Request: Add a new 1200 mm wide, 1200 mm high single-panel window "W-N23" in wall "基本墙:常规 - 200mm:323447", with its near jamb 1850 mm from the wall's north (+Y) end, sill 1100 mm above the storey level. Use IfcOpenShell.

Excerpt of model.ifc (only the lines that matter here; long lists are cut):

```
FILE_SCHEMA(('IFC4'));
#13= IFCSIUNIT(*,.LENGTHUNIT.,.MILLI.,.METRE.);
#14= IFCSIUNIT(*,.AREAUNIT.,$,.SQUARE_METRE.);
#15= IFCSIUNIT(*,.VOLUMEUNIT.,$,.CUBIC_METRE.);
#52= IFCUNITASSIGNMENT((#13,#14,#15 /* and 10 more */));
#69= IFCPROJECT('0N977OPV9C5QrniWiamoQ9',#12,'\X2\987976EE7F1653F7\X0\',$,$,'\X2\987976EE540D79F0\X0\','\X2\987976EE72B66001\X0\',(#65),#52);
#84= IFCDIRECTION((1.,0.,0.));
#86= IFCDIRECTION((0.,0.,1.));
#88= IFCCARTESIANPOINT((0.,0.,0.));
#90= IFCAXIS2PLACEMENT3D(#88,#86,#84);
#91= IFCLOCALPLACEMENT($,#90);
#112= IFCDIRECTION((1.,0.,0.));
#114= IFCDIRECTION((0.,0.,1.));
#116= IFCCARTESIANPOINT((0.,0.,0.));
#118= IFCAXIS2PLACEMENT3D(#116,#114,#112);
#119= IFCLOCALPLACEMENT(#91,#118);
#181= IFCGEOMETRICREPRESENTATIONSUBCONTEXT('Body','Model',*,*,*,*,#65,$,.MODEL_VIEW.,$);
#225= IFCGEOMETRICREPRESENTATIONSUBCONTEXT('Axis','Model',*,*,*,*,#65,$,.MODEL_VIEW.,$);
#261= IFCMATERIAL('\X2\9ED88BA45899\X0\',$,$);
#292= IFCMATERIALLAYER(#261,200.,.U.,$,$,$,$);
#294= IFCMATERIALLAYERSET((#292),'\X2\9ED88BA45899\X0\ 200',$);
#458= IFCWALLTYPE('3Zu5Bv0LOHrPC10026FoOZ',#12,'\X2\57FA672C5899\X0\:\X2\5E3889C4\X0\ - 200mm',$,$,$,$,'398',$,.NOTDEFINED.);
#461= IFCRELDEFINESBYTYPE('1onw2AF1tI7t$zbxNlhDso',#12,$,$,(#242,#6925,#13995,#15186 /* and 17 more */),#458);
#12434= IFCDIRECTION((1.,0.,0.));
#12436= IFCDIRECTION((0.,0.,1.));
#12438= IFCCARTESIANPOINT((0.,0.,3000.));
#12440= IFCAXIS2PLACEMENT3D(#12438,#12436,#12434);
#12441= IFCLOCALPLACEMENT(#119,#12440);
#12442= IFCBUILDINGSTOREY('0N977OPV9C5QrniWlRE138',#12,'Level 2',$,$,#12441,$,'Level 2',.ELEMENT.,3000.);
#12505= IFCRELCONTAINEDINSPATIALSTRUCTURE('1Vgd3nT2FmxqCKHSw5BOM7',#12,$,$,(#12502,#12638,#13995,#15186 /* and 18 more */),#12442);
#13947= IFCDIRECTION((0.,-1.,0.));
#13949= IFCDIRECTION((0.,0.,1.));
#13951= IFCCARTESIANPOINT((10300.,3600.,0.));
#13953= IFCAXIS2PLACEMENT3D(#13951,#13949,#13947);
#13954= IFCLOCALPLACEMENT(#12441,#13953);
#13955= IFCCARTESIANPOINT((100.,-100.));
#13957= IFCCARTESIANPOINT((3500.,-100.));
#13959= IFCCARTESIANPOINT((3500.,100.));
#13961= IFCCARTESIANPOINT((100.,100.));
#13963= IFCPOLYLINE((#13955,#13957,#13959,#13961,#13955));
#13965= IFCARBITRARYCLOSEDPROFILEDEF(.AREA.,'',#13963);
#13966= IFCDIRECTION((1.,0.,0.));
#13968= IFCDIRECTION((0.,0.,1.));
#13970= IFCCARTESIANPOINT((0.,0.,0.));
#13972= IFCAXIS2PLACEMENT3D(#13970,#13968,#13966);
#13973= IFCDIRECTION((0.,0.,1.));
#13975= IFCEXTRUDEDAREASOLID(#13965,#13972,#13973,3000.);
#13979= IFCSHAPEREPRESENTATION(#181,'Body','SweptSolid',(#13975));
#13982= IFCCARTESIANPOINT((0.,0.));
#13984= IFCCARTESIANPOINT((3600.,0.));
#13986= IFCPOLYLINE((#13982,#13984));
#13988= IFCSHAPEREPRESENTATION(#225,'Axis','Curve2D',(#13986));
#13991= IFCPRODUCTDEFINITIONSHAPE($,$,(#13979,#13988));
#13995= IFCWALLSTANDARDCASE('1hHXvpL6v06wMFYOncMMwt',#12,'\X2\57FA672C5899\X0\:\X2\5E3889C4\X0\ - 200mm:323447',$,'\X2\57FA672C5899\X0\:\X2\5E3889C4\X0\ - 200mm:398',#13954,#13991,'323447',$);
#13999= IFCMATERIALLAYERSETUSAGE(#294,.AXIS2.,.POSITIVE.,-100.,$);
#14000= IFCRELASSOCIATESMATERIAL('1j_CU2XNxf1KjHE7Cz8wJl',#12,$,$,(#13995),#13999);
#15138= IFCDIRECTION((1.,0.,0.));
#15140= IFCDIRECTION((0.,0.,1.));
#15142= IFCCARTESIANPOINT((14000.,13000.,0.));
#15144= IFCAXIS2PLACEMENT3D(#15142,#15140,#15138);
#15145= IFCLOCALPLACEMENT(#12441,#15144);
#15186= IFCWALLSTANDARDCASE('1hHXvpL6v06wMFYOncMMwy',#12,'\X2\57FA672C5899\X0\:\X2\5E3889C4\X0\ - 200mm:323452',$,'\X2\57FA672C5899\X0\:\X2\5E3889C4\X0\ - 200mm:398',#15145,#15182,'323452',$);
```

```python
import numpy as np
import ifcopenshell
import ifcopenshell.api.feature
import ifcopenshell.api.geometry
import ifcopenshell.api.root
import ifcopenshell.api.spatial
import ifcopenshell.geom
import ifcopenshell.util.element
import ifcopenshell.util.placement
import ifcopenshell.util.representation
import ifcopenshell.util.shape
import ifcopenshell.util.unit

model = ifcopenshell.open("model.ifc")
unit_scale = ifcopenshell.util.unit.calculate_unit_scale(model)
settings = ifcopenshell.geom.settings()


def volume(element):
    """Net volume in cubic metres, openings subtracted."""
    shape = ifcopenshell.geom.create_shape(settings, element)
    return ifcopenshell.util.shape.get_volume(shape.geometry)


wall = model.by_guid("1hHXvpL6v06wMFYOncMMwt")
storey = ifcopenshell.util.element.get_container(wall, ifc_class="IfcBuildingStorey")
context = ifcopenshell.util.representation.get_context(model, "Model", "Body", "MODEL_VIEW")
before = volume(wall)

width, height, from_end, sill = 1.2, 1.2, 1.85, 1.1  # metres

# The wall runs along its own X axis, and the end named is its -X end.
wall_shape = ifcopenshell.geom.create_shape(settings, wall)
x, y, z = ifcopenshell.util.shape.get_vertices(wall_shape.geometry).T
start = x.min() + from_end
face, thickness = float(y.min()), float(y.max() - y.min())
wall_matrix = ifcopenshell.util.placement.get_local_placement(wall.ObjectPlacement)
level = ifcopenshell.util.placement.get_local_placement(storey.ObjectPlacement)[2, 3]


def in_wall(x, y):
    """Placement at x, y metres in the wall's axes, at sill height."""
    matrix = wall_matrix.copy()
    matrix[:, 3] = wall_matrix @ np.array([x / unit_scale, y / unit_scale, 0.0, 1.0])
    matrix[2, 3] = level + sill / unit_scale
    return matrix


# Opening: a box that overshoots both wall faces by 50 mm.
opening = ifcopenshell.api.root.create_entity(model, ifc_class="IfcOpeningElement", predefined_type="OPENING")
box = ifcopenshell.api.geometry.add_wall_representation(
    model, context=context, length=width, height=height, thickness=thickness + 0.1
)
ifcopenshell.api.geometry.assign_representation(model, product=opening, representation=box)
ifcopenshell.api.geometry.edit_object_placement(model, product=opening, matrix=in_wall(start, face - 0.05), is_si=False)
ifcopenshell.api.feature.add_feature(model, feature=opening, element=wall)

window = ifcopenshell.api.root.create_entity(model, ifc_class="IfcWindow", name="W-N23", predefined_type="WINDOW")
window.OverallWidth, window.OverallHeight = width / unit_scale, height / unit_scale
window.PartitioningType = "SINGLE_PANEL"
body = ifcopenshell.api.geometry.add_window_representation(
    model,
    context=context,
    overall_width=window.OverallWidth,
    overall_height=window.OverallHeight,
    partition_type="SINGLE_PANEL",
)
ifcopenshell.api.geometry.assign_representation(model, product=window, representation=body)
ifcopenshell.api.spatial.assign_container(model, products=[window], relating_structure=storey)
ifcopenshell.api.feature.add_filling(model, opening=opening, element=window)

# Centre the window in the wall's thickness.
ifcopenshell.api.geometry.edit_object_placement(model, product=window, matrix=in_wall(start, face), is_si=False)
window_shape = ifcopenshell.geom.create_shape(settings, window)
depth = ifcopenshell.util.shape.get_vertices(window_shape.geometry)[:, 1]
offset = face + thickness / 2 - (depth.min() + depth.max()) / 2
ifcopenshell.api.geometry.edit_object_placement(model, product=window, matrix=in_wall(start, offset), is_si=False)

after = volume(wall)

print(f"wall volume {before:.3f} -> {after:.3f} m3")

model.write("model_edited.ifc")
```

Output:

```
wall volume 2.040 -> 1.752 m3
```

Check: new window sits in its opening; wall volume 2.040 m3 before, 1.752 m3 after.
